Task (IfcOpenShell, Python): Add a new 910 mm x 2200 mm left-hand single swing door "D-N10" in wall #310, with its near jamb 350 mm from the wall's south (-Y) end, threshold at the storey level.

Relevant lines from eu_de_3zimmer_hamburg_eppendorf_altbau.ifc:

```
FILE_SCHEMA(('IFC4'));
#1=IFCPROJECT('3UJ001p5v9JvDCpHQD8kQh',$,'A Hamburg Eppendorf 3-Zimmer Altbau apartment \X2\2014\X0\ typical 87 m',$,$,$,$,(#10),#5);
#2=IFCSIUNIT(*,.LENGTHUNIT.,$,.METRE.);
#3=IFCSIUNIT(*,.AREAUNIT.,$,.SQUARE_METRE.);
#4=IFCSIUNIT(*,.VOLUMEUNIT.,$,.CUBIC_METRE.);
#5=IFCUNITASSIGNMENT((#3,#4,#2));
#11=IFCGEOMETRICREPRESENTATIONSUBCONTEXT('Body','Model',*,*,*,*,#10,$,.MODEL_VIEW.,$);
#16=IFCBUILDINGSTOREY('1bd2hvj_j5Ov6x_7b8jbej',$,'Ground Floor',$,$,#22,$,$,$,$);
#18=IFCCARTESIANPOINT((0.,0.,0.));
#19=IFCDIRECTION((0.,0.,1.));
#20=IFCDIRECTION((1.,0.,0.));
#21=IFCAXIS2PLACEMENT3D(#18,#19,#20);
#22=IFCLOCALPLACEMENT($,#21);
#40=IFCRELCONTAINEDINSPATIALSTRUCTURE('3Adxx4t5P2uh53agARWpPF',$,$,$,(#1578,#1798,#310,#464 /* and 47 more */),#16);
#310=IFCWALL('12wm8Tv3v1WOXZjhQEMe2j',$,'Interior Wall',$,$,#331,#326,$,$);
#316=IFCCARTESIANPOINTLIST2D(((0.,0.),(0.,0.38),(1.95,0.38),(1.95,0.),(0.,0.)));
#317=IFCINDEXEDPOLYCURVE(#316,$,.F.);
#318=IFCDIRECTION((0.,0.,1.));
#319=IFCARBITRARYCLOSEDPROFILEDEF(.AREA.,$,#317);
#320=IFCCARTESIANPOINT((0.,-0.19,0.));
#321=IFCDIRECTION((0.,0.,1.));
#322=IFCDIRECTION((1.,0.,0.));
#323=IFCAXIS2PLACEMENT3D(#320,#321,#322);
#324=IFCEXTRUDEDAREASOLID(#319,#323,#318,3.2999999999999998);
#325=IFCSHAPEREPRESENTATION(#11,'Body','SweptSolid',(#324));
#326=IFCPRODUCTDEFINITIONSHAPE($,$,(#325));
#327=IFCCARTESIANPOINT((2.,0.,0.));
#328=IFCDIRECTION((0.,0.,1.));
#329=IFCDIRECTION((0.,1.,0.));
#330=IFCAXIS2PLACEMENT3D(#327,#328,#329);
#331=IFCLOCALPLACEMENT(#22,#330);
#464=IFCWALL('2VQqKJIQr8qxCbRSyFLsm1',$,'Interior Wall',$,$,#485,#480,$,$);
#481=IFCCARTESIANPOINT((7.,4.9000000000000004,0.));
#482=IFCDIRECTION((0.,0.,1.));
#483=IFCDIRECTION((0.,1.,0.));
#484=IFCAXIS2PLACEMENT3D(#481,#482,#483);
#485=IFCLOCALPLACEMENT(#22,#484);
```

```python
import numpy as np
import ifcopenshell
import ifcopenshell.api.feature
import ifcopenshell.api.geometry
import ifcopenshell.api.root
import ifcopenshell.api.spatial
import ifcopenshell.geom
import ifcopenshell.util.element
import ifcopenshell.util.placement
import ifcopenshell.util.representation
import ifcopenshell.util.shape
import ifcopenshell.util.unit

model = ifcopenshell.open("eu_de_3zimmer_hamburg_eppendorf_altbau.ifc")
unit_scale = ifcopenshell.util.unit.calculate_unit_scale(model)
settings = ifcopenshell.geom.settings()


def volume(element):
    """Net volume in cubic metres, openings subtracted."""
    shape = ifcopenshell.geom.create_shape(settings, element)
    return ifcopenshell.util.shape.get_volume(shape.geometry)


wall = model.by_id(310)
storey = ifcopenshell.util.element.get_container(wall, ifc_class="IfcBuildingStorey")
context = ifcopenshell.util.representation.get_context(model, "Model", "Body", "MODEL_VIEW")
before = volume(wall)

width, height, from_end, sill = 0.91, 2.2, 0.35, 0.0  # metres

# The wall runs along its own X axis, and the end named is its -X end.
wall_shape = ifcopenshell.geom.create_shape(settings, wall)
x, y, z = ifcopenshell.util.shape.get_vertices(wall_shape.geometry).T
start = x.min() + from_end
face, thickness = float(y.min()), float(y.max() - y.min())
wall_matrix = ifcopenshell.util.placement.get_local_placement(wall.ObjectPlacement)
level = ifcopenshell.util.placement.get_local_placement(storey.ObjectPlacement)[2, 3]


def in_wall(x, y):
    """Placement at x, y metres in the wall's axes, at sill height."""
    matrix = wall_matrix.copy()
    matrix[:, 3] = wall_matrix @ np.array([x / unit_scale, y / unit_scale, 0.0, 1.0])
    matrix[2, 3] = level + sill / unit_scale
    return matrix


# Opening: a box that overshoots both wall faces by 50 mm.
opening = ifcopenshell.api.root.create_entity(model, ifc_class="IfcOpeningElement", predefined_type="OPENING")
box = ifcopenshell.api.geometry.add_wall_representation(
    model, context=context, length=width, height=height, thickness=thickness + 0.1
)
ifcopenshell.api.geometry.assign_representation(model, product=opening, representation=box)
ifcopenshell.api.geometry.edit_object_placement(model, product=opening, matrix=in_wall(start, face - 0.05), is_si=False)
ifcopenshell.api.feature.add_feature(model, feature=opening, element=wall)

door = ifcopenshell.api.root.create_entity(model, ifc_class="IfcDoor", name="D-N10", predefined_type="DOOR")
door.OverallWidth, door.OverallHeight = width / unit_scale, height / unit_scale
door.OperationType = "SINGLE_SWING_LEFT"
body = ifcopenshell.api.geometry.add_door_representation(
    model,
    context=context,
    overall_width=door.OverallWidth,
    overall_height=door.OverallHeight,
    operation_type="SINGLE_SWING_LEFT",
    lining_properties={"LiningDepth": thickness / unit_scale, "ThresholdDepth": thickness / unit_scale},
)
ifcopenshell.api.geometry.assign_representation(model, product=door, representation=body)
ifcopenshell.api.spatial.assign_container(model, products=[door], relating_structure=storey)
ifcopenshell.api.feature.add_filling(model, opening=opening, element=door)

# The lining spans the wall, so the door starts at the wall face.
ifcopenshell.api.geometry.edit_object_placement(model, product=door, matrix=in_wall(start, face), is_si=False)

after = volume(wall)

print(f"wall volume {before:.3f} -> {after:.3f} m3")

model.write("eu_de_3zimmer_hamburg_eppendorf_altbau_rev.ifc")
```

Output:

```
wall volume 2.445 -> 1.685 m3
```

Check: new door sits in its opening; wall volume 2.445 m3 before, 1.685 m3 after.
